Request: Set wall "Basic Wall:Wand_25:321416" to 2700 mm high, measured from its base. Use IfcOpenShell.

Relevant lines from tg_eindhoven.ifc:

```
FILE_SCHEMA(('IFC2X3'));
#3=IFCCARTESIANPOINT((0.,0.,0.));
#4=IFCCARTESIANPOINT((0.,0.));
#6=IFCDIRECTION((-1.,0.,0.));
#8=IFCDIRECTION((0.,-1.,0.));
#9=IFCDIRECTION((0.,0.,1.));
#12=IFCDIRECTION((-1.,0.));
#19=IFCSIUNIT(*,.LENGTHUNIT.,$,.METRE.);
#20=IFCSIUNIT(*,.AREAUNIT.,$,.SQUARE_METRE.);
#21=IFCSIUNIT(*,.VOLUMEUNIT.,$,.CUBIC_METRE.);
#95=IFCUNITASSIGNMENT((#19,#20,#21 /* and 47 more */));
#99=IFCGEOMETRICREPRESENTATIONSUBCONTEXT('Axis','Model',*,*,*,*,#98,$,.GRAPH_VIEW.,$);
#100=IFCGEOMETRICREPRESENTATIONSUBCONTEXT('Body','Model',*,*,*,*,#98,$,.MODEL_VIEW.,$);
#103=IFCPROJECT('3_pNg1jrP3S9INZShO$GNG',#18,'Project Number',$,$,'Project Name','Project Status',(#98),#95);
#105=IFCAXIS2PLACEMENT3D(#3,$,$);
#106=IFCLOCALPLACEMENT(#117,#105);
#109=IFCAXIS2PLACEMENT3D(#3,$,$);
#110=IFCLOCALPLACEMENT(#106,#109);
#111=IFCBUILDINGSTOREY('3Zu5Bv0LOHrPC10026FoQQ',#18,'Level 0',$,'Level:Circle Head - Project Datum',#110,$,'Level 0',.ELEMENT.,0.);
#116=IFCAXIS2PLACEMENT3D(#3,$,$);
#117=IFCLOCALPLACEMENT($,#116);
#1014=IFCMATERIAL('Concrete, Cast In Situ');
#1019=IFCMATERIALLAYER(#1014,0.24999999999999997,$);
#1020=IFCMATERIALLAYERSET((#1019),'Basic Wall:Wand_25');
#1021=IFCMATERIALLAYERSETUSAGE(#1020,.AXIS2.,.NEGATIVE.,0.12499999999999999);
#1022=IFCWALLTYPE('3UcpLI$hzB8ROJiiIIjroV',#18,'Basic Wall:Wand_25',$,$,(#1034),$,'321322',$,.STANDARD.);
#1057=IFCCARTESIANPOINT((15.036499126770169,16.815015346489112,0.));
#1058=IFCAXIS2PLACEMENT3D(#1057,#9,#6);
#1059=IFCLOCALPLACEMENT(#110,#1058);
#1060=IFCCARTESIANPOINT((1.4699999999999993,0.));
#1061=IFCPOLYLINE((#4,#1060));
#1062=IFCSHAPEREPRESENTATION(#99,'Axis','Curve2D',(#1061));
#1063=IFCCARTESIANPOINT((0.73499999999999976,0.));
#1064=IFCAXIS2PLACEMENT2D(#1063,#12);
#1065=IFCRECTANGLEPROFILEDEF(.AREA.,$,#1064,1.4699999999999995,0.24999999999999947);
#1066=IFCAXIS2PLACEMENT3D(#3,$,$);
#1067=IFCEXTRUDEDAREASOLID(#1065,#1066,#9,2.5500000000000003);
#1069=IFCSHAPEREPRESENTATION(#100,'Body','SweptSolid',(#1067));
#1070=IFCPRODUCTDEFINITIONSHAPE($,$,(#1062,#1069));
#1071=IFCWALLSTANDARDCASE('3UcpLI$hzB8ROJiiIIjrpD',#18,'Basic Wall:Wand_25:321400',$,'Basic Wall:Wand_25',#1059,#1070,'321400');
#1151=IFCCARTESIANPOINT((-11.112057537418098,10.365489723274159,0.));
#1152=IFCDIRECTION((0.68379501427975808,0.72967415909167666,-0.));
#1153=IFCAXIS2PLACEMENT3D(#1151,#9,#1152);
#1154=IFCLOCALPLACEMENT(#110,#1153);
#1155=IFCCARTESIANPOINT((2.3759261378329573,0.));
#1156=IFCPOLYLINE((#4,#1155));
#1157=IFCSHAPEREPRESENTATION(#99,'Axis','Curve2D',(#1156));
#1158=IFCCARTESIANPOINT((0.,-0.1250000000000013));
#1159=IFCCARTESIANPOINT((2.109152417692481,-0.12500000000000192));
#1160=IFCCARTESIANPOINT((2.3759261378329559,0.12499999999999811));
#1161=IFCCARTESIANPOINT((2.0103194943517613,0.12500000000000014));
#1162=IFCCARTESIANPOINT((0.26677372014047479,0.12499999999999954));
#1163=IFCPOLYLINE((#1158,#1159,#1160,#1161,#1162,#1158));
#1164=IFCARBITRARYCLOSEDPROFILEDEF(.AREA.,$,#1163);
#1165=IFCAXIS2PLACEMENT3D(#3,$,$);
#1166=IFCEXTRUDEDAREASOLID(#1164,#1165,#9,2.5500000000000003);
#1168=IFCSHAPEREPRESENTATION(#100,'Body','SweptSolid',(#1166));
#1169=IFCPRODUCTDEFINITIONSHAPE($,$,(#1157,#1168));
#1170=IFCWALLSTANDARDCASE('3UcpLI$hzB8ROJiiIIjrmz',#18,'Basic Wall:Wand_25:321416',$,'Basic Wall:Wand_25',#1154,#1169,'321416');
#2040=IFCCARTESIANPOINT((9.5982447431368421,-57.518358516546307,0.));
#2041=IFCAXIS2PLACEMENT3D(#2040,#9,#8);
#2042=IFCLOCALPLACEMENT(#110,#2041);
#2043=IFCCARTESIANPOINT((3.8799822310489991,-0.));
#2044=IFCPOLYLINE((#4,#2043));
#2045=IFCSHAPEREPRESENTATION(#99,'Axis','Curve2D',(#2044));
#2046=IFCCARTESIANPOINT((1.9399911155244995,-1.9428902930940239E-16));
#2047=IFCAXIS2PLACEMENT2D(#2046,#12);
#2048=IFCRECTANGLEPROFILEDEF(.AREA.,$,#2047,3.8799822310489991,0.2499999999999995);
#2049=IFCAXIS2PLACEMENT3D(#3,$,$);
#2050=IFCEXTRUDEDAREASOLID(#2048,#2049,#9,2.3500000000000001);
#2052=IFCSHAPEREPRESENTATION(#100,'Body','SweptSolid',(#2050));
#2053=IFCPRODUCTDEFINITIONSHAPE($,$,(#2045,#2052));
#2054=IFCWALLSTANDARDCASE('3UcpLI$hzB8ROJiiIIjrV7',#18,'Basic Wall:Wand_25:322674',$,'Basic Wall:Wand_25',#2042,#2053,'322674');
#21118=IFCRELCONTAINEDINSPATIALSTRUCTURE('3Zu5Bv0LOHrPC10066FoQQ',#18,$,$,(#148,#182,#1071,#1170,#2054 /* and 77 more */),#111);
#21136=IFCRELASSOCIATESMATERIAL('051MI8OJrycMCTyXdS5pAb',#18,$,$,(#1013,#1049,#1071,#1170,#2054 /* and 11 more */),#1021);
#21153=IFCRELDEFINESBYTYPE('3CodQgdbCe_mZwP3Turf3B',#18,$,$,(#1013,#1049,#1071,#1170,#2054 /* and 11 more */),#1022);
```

```python
import ifcopenshell
import ifcopenshell.geom
import ifcopenshell.util.representation
import ifcopenshell.util.shape

model = ifcopenshell.open("tg_eindhoven.ifc")
settings = ifcopenshell.geom.settings()


def volume(element):
    """Net volume in cubic metres, openings subtracted."""
    shape = ifcopenshell.geom.create_shape(settings, element)
    return ifcopenshell.util.shape.get_volume(shape.geometry)


wall = model.by_guid("3UcpLI$hzB8ROJiiIIjrmz")
before = volume(wall)

body = ifcopenshell.util.representation.get_representation(wall, "Model", "Body")
solid = body.Items[0]
old_height = solid.Depth
solid.Depth = 2.7
after = volume(wall)

print(f"height {old_height:g} -> {solid.Depth:g}, volume {before:.3f} -> {after:.3f} m3")

model.write("tg_eindhoven_rev.ifc")
```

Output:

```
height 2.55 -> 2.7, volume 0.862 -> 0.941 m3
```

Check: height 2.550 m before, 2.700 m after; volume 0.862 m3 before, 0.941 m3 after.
